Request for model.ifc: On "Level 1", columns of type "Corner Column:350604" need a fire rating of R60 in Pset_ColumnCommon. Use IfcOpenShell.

First a look at what the model holds.

```python
import ifcopenshell
import ifcopenshell.util.element

model = ifcopenshell.open("model.ifc")
print(model.schema)
storey = next(s for s in model.by_type("IfcBuildingStorey") if s.Name == "Level 1")
columns = [e for e in ifcopenshell.util.element.get_decomposition(storey) if e.is_a("IfcColumn")]
seen = {}
for e in columns:
    element_type = ifcopenshell.util.element.get_type(e)
    key = (element_type.Name if element_type != e and element_type else None, ifcopenshell.util.element.get_pset(e, "Pset_ColumnCommon", "FireRating"))
    seen[key] = seen.get(key, 0) + 1
for (name, value), count in sorted(seen.items(), key=str):
    print(count, "x", name, "|", value)
```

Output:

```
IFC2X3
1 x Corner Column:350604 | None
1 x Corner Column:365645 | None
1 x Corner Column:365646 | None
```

```python
import ifcopenshell
import ifcopenshell.api.pset
import ifcopenshell.util.element

model = ifcopenshell.open("model.ifc")

storey = next(s for s in model.by_type("IfcBuildingStorey") if s.Name == "Level 1")
columns = [e for e in ifcopenshell.util.element.get_decomposition(storey) if e.is_a("IfcColumn")]

count = 0
for e in columns:
    element_type = ifcopenshell.util.element.get_type(e)
    if element_type in (None, e) or element_type.Name != "Corner Column:350604":
        continue
    # add_pset returns the element's existing set when there is one.
    pset = ifcopenshell.api.pset.add_pset(model, product=e, name="Pset_ColumnCommon")
    ifcopenshell.api.pset.edit_pset(model, pset=pset, properties={"FireRating": "R60"})
    count += 1

print(count, "columns updated")

model.write("model_rev.ifc")
```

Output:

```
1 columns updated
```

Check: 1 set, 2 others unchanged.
